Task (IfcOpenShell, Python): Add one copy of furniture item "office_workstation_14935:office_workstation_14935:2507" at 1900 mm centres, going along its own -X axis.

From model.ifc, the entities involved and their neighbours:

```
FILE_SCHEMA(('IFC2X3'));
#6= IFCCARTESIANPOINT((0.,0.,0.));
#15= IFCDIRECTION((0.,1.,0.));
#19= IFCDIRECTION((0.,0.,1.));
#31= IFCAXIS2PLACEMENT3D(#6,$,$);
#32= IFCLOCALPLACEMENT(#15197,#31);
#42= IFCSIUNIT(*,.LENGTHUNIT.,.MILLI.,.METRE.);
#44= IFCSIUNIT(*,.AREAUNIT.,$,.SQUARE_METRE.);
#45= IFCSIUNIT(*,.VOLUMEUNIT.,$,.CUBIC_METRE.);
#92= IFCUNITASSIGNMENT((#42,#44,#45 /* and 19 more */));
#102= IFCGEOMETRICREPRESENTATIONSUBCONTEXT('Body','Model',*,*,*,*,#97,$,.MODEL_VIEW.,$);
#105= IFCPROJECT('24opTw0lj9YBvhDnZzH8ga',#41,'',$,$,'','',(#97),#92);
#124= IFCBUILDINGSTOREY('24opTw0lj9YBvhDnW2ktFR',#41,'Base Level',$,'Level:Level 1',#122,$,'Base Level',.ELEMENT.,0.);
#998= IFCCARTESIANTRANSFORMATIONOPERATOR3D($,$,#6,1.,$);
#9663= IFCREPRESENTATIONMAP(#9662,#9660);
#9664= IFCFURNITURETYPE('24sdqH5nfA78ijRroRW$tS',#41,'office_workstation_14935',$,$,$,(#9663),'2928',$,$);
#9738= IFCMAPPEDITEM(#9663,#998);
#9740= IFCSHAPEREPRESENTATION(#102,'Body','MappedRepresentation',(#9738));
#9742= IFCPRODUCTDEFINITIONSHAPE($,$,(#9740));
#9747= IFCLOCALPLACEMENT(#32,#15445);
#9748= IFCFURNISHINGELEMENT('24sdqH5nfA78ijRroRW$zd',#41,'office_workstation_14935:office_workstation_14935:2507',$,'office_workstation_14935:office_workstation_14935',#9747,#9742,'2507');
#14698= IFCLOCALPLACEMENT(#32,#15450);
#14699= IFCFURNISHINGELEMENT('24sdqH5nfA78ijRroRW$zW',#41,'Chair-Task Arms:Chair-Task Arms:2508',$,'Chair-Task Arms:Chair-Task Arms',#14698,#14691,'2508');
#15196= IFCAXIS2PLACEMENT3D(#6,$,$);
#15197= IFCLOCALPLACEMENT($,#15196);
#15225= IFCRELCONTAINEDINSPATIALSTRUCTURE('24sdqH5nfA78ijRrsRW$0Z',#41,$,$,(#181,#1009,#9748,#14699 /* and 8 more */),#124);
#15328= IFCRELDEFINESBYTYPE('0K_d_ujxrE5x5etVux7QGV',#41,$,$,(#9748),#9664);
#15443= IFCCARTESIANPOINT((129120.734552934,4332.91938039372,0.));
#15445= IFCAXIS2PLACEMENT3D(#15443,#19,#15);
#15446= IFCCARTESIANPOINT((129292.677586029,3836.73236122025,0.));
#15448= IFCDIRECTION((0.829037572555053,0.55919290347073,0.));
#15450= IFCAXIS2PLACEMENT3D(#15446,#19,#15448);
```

```python
import ifcopenshell
import ifcopenshell.api.geometry
import ifcopenshell.api.root
import ifcopenshell.util.element
import ifcopenshell.util.placement
import ifcopenshell.util.unit

model = ifcopenshell.open("model.ifc")
unit_scale = ifcopenshell.util.unit.calculate_unit_scale(model)


def reuse_history(source, copy):
    """copy_class also copies each property set's owner history, people and application; keep the originals."""
    for rel in copy.IsDefinedBy:
        if rel.is_a("IfcRelDefinesByProperties") and (history := rel.RelatingPropertyDefinition.OwnerHistory):
            rel.RelatingPropertyDefinition.OwnerHistory = source.OwnerHistory
            ifcopenshell.util.element.remove_deep2(model, history)


source = model.by_guid("24sdqH5nfA78ijRroRW$zd")
base = ifcopenshell.util.placement.get_local_placement(source.ObjectPlacement)
step = -base[:3, 0] * 1.9 / unit_scale

for i in range(1, 2):
    copy = ifcopenshell.api.root.copy_class(model, product=source)
    copy.Representation = ifcopenshell.util.element.copy_deep(
        model, source.Representation, exclude=["IfcGeometricRepresentationContext", "IfcRepresentationMap"]
    )
    copy.Name = "office_workstation_14935:office_workstation_14935"
    copy.Tag = None
    reuse_history(source, copy)
    matrix = base.copy()
    matrix[:3, 3] += i * step
    print("added at", matrix[:3, 3].round(3) + 0.0)
    ifcopenshell.api.geometry.edit_object_placement(model, product=copy, matrix=matrix, is_si=False)

model.write("model_updated.ifc")
```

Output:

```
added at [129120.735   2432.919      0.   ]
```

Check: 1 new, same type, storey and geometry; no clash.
